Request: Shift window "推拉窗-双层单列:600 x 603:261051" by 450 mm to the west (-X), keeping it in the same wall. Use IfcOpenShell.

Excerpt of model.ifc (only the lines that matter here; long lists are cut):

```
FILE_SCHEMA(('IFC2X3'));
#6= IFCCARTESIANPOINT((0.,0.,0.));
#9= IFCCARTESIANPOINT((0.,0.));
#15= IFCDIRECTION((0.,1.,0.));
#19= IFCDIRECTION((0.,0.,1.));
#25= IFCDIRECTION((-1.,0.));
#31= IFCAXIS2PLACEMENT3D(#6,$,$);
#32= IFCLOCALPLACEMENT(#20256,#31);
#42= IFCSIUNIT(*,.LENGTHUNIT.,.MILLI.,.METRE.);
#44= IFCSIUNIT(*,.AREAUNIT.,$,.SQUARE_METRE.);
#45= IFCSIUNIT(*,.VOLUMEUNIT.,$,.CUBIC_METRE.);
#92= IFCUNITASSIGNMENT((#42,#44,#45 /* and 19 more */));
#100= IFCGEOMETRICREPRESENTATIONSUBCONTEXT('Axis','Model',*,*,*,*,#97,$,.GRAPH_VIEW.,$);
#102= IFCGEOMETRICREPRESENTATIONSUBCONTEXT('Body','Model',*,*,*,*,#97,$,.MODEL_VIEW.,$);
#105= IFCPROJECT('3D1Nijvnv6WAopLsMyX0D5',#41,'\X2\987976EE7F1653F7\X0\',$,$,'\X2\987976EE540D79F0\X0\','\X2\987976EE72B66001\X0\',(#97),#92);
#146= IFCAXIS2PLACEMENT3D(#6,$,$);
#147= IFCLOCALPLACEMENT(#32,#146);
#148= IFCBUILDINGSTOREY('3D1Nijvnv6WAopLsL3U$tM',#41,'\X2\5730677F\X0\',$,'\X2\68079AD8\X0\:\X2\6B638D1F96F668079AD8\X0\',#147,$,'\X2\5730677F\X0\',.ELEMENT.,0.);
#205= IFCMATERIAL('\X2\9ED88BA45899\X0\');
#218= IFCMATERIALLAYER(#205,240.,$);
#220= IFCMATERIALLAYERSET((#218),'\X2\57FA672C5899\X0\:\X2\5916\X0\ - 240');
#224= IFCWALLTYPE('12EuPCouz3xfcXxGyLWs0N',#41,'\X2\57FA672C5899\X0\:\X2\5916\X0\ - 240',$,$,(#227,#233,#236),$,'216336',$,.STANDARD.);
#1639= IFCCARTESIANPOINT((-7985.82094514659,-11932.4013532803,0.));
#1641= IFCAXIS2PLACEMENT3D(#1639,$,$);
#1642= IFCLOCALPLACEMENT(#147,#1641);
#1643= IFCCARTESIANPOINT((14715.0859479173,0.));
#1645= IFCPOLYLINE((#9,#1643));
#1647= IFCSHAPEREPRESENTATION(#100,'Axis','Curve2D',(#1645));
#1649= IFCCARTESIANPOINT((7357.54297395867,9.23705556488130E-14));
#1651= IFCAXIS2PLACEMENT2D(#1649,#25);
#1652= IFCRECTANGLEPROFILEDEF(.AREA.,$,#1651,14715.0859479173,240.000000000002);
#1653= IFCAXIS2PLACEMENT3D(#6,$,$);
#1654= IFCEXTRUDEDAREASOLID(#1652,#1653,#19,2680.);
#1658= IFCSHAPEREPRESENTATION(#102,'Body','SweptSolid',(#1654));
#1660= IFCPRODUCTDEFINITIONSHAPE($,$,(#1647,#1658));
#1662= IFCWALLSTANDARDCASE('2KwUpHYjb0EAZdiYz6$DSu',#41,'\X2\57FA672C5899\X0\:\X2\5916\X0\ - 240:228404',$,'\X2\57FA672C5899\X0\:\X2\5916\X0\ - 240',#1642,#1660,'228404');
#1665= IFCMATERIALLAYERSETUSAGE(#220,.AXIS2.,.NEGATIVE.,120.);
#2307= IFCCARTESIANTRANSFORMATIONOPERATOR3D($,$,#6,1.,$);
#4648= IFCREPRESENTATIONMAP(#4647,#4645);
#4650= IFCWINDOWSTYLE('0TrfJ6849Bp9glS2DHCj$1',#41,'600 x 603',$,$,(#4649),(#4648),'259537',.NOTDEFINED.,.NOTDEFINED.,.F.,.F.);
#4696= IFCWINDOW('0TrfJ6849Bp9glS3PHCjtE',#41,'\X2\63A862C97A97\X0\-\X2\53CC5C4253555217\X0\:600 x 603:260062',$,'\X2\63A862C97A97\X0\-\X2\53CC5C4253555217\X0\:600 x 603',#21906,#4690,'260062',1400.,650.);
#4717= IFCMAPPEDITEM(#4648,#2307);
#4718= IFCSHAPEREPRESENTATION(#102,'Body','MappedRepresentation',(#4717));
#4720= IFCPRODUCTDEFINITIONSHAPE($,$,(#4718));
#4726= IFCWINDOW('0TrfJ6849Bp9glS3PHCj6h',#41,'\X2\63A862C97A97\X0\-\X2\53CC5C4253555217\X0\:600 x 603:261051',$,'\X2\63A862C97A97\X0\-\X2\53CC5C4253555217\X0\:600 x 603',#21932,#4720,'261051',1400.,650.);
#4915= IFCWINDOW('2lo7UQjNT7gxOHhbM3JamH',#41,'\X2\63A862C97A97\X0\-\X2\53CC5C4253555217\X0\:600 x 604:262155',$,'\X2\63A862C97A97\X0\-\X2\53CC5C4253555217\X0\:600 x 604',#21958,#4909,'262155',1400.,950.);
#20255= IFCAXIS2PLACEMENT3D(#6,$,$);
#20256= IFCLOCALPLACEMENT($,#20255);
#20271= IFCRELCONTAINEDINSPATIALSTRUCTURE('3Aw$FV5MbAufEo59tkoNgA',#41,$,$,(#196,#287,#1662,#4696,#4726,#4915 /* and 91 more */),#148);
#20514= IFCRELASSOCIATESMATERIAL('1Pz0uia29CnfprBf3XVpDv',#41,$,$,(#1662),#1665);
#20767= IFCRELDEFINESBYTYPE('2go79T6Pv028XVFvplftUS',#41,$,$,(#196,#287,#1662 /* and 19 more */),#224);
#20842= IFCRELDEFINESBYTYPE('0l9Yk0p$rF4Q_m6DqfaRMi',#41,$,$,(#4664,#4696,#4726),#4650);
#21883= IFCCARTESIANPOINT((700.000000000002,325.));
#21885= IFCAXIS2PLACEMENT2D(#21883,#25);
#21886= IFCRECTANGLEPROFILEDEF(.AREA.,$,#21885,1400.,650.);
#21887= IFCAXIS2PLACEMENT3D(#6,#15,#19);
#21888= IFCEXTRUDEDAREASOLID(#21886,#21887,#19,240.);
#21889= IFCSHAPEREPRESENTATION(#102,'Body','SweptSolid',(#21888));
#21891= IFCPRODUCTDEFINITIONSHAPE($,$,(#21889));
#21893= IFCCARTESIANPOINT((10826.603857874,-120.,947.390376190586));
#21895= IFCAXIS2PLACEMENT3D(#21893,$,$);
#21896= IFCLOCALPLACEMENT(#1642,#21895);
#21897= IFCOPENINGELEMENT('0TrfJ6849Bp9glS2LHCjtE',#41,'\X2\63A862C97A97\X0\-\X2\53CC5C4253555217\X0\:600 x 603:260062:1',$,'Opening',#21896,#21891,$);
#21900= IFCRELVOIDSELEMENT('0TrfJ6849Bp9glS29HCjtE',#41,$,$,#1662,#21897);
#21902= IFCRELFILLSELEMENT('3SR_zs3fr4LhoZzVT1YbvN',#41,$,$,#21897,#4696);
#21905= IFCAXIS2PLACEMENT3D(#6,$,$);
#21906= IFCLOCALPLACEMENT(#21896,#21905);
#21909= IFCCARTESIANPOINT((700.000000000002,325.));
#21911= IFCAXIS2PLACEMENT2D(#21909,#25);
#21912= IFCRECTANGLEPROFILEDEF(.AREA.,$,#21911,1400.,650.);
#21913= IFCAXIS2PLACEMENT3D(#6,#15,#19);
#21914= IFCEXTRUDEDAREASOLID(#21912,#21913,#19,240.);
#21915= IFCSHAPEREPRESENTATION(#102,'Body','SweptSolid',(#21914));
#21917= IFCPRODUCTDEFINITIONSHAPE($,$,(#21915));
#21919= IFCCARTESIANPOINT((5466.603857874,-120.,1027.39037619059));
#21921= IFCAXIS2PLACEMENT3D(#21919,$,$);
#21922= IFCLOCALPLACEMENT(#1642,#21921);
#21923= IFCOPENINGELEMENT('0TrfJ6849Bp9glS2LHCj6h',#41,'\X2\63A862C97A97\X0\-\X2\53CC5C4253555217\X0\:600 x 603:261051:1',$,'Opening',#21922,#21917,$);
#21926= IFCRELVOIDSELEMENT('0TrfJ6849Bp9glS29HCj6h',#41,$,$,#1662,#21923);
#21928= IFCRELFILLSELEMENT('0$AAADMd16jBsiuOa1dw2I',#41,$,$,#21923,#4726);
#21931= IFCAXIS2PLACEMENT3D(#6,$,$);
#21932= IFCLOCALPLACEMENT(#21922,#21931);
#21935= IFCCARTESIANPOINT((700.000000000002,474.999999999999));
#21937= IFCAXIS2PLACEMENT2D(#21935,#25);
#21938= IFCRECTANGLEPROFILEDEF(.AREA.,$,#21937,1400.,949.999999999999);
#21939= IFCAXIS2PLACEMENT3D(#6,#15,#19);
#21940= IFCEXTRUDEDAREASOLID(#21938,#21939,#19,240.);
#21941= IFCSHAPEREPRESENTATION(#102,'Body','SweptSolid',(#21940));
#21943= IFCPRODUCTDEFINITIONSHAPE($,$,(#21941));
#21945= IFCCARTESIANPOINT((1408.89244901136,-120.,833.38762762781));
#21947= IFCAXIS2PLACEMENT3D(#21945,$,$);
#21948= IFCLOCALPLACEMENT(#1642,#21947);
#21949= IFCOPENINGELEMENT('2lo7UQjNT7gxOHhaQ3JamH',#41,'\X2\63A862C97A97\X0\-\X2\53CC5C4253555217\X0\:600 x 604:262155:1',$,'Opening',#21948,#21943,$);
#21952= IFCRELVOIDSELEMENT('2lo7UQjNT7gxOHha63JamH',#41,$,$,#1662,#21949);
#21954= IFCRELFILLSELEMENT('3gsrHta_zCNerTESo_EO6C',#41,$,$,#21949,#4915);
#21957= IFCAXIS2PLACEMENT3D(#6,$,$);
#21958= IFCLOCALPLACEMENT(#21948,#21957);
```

```python
import ifcopenshell
import ifcopenshell.api.geometry
import ifcopenshell.util.placement

model = ifcopenshell.open("model.ifc")

window = model.by_id(4726)
opening = window.FillsVoids[0].RelatingOpeningElement
wall = opening.VoidsElements[0].RelatingBuildingElement

wall_matrix = ifcopenshell.util.placement.get_local_placement(wall.ObjectPlacement)
shift = wall_matrix[:3, 0] * -450.0
before = ifcopenshell.util.placement.get_local_placement(window.ObjectPlacement)[:3, 3].copy()

# The window is placed relative to its opening, so it follows when the opening moves.
matrix = ifcopenshell.util.placement.get_local_placement(opening.ObjectPlacement)
matrix[:3, 3] += shift
ifcopenshell.api.geometry.edit_object_placement(
    model, product=opening, matrix=matrix, is_si=False, should_transform_children=True
)

after = ifcopenshell.util.placement.get_local_placement(window.ObjectPlacement)[:3, 3]
print("window moved by", (after - before).round(3) + 0.0)

model.write("model-out.ifc")
```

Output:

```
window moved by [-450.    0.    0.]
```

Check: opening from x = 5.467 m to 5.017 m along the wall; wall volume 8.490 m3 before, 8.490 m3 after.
